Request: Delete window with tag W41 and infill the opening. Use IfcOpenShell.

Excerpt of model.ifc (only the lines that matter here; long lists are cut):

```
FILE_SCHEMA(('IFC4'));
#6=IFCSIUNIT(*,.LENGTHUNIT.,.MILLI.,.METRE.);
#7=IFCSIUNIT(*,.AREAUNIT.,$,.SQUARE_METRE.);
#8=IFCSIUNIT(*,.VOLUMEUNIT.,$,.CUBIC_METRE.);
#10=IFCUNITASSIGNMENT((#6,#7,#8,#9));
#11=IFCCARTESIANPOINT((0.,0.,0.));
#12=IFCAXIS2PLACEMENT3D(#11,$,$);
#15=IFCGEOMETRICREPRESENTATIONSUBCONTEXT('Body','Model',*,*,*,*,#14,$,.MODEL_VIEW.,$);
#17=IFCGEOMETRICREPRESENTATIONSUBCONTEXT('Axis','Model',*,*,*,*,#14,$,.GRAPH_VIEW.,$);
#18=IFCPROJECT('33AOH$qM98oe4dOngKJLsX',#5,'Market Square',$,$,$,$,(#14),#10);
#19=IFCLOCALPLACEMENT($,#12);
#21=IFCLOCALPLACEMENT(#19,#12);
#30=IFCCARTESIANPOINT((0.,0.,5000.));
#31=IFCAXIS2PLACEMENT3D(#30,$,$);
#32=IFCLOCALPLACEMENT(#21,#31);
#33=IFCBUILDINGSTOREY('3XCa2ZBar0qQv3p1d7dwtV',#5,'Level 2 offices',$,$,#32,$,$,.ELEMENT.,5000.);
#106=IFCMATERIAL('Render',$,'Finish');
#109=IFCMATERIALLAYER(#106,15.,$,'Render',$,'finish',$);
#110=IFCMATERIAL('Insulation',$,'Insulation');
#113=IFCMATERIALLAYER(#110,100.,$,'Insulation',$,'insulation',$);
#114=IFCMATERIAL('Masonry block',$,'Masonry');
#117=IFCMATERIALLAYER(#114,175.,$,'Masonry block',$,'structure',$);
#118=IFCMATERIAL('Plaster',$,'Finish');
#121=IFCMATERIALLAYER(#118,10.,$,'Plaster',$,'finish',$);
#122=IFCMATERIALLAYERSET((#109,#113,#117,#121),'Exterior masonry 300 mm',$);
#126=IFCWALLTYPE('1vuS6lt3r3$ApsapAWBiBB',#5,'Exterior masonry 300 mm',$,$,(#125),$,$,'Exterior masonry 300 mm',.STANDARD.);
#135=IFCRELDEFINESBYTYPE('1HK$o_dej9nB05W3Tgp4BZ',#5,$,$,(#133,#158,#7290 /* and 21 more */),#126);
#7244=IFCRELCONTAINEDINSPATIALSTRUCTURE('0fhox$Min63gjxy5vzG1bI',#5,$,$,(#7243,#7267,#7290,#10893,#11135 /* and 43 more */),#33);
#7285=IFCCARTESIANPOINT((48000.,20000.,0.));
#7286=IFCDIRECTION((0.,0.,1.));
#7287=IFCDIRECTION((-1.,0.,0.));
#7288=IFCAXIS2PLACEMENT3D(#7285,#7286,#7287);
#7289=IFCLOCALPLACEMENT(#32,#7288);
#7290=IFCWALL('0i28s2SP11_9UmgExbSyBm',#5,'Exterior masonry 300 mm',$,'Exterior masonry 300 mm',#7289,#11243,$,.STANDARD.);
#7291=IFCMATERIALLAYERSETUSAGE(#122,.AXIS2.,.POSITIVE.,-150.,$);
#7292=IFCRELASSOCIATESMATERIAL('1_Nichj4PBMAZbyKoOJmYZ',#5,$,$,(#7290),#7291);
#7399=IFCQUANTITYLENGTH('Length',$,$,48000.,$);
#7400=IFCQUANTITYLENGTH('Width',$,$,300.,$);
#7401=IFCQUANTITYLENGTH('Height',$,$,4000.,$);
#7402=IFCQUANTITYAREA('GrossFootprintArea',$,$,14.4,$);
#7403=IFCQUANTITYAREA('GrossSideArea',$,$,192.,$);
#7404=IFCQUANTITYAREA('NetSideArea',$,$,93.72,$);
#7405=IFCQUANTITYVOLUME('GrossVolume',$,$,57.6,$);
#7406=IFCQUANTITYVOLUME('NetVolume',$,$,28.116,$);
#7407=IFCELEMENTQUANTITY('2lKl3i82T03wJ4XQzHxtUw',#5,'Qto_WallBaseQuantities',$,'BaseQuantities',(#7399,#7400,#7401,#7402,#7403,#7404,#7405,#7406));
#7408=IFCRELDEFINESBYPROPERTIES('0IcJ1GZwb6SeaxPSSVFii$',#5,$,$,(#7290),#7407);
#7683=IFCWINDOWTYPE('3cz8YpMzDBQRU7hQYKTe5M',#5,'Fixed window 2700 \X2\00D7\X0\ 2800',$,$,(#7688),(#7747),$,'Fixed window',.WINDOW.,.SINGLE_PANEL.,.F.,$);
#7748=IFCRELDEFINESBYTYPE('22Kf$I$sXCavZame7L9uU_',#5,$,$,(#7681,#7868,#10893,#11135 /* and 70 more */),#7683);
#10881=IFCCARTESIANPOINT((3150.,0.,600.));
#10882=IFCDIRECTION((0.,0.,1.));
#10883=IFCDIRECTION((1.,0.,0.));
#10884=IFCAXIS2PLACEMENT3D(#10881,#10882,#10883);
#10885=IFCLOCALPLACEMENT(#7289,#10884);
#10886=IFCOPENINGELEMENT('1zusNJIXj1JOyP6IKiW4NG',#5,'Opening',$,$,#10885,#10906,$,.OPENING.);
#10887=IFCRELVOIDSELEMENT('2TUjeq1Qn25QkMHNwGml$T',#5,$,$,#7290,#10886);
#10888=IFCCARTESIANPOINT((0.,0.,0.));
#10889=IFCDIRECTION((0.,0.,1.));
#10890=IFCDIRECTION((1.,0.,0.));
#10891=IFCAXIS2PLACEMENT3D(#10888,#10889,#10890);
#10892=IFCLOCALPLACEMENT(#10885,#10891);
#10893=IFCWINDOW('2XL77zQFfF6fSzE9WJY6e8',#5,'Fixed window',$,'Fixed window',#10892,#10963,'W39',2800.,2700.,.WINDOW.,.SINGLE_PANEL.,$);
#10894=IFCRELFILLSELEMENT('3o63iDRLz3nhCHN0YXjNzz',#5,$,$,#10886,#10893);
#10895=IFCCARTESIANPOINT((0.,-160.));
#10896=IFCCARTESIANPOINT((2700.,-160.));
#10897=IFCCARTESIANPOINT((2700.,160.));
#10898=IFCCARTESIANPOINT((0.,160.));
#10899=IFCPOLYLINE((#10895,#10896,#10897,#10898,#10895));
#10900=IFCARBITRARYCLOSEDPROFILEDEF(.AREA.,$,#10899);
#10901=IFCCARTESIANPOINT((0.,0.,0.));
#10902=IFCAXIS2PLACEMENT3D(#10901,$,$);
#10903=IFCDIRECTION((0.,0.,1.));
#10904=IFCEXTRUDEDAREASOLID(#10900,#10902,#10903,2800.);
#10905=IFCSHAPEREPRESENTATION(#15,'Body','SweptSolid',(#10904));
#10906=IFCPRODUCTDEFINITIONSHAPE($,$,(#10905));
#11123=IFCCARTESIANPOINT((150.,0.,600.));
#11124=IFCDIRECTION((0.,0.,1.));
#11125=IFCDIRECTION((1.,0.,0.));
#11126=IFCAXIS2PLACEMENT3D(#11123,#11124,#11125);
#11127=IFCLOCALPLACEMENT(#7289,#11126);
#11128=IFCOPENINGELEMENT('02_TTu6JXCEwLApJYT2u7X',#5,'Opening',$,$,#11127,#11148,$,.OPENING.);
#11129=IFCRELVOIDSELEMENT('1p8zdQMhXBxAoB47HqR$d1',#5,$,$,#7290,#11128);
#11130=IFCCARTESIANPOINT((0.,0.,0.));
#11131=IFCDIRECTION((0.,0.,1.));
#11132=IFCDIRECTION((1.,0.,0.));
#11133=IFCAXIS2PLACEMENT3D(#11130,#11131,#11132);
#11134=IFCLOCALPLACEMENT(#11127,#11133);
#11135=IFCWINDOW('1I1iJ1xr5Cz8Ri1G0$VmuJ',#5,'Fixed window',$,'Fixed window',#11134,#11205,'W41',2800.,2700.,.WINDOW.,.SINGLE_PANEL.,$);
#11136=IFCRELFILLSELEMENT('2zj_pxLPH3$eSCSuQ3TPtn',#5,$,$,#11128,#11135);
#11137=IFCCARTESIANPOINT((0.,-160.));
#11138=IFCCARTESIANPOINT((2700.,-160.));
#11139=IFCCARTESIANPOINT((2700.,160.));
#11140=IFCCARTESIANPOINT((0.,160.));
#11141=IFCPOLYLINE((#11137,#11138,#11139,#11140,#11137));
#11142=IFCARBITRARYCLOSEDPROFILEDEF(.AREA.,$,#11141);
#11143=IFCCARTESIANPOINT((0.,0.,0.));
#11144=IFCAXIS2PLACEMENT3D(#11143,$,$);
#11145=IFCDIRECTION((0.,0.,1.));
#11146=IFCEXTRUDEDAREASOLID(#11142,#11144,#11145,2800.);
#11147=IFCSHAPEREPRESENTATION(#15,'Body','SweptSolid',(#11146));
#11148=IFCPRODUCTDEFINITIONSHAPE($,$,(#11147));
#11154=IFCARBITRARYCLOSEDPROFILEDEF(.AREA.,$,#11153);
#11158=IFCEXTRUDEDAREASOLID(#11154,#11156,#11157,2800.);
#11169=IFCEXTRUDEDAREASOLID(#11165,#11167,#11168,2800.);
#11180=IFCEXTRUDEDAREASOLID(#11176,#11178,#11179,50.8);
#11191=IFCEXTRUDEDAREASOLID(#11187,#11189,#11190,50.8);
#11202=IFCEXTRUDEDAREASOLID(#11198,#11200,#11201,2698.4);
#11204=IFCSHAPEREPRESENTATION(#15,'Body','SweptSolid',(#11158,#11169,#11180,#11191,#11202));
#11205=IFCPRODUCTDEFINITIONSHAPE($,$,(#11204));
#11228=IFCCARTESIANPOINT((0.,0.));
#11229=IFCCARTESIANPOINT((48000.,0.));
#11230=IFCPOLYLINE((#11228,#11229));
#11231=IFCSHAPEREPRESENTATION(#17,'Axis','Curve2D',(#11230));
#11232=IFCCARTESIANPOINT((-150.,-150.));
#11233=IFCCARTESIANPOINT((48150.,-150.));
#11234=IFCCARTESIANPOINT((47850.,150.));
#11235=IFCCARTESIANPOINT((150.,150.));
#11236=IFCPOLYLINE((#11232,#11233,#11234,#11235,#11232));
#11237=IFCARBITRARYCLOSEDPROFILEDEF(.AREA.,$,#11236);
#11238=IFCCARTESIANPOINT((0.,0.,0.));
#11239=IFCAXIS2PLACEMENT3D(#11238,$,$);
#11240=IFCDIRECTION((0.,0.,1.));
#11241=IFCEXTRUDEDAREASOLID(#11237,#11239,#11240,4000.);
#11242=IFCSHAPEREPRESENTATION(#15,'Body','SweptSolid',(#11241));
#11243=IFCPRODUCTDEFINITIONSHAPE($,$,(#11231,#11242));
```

```python
import ifcopenshell
import ifcopenshell.api.feature
import ifcopenshell.api.pset
import ifcopenshell.api.root
import ifcopenshell.geom
import ifcopenshell.util.element
import ifcopenshell.util.shape
import ifcopenshell.util.unit

model = ifcopenshell.open("model.ifc")
area_scale = ifcopenshell.util.unit.calculate_unit_scale(model, "AREAUNIT")
volume_scale = ifcopenshell.util.unit.calculate_unit_scale(model, "VOLUMEUNIT")
settings = ifcopenshell.geom.settings()


def volume(element):
    """Net volume in cubic metres, openings subtracted."""
    shape = ifcopenshell.geom.create_shape(settings, element)
    return ifcopenshell.util.shape.get_volume(shape.geometry)


window = model.by_guid("1I1iJ1xr5Cz8Ri1G0$VmuJ")
opening = window.FillsVoids[0].RelatingOpeningElement
wall = opening.VoidsElements[0].RelatingBuildingElement
before = volume(wall)

ifcopenshell.api.root.remove_product(model, product=window)
ifcopenshell.api.feature.remove_feature(model, feature=opening)

after = volume(wall)
thickness = 0.3  # wall thickness in metres

# Update the wall's stored quantities.
qto = model.by_id(ifcopenshell.util.element.get_pset(wall, "Qto_WallBaseQuantities", should_inherit=False)["id"])
ifcopenshell.api.pset.edit_qto(model, qto=qto, properties={
    "NetSideArea": after / thickness / area_scale,
    "NetVolume": after / volume_scale,
})

print(f"wall volume {before:.3f} -> {after:.3f} m3")

model.write("model_v2.ifc")
```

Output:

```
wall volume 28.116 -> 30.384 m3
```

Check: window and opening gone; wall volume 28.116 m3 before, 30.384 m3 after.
